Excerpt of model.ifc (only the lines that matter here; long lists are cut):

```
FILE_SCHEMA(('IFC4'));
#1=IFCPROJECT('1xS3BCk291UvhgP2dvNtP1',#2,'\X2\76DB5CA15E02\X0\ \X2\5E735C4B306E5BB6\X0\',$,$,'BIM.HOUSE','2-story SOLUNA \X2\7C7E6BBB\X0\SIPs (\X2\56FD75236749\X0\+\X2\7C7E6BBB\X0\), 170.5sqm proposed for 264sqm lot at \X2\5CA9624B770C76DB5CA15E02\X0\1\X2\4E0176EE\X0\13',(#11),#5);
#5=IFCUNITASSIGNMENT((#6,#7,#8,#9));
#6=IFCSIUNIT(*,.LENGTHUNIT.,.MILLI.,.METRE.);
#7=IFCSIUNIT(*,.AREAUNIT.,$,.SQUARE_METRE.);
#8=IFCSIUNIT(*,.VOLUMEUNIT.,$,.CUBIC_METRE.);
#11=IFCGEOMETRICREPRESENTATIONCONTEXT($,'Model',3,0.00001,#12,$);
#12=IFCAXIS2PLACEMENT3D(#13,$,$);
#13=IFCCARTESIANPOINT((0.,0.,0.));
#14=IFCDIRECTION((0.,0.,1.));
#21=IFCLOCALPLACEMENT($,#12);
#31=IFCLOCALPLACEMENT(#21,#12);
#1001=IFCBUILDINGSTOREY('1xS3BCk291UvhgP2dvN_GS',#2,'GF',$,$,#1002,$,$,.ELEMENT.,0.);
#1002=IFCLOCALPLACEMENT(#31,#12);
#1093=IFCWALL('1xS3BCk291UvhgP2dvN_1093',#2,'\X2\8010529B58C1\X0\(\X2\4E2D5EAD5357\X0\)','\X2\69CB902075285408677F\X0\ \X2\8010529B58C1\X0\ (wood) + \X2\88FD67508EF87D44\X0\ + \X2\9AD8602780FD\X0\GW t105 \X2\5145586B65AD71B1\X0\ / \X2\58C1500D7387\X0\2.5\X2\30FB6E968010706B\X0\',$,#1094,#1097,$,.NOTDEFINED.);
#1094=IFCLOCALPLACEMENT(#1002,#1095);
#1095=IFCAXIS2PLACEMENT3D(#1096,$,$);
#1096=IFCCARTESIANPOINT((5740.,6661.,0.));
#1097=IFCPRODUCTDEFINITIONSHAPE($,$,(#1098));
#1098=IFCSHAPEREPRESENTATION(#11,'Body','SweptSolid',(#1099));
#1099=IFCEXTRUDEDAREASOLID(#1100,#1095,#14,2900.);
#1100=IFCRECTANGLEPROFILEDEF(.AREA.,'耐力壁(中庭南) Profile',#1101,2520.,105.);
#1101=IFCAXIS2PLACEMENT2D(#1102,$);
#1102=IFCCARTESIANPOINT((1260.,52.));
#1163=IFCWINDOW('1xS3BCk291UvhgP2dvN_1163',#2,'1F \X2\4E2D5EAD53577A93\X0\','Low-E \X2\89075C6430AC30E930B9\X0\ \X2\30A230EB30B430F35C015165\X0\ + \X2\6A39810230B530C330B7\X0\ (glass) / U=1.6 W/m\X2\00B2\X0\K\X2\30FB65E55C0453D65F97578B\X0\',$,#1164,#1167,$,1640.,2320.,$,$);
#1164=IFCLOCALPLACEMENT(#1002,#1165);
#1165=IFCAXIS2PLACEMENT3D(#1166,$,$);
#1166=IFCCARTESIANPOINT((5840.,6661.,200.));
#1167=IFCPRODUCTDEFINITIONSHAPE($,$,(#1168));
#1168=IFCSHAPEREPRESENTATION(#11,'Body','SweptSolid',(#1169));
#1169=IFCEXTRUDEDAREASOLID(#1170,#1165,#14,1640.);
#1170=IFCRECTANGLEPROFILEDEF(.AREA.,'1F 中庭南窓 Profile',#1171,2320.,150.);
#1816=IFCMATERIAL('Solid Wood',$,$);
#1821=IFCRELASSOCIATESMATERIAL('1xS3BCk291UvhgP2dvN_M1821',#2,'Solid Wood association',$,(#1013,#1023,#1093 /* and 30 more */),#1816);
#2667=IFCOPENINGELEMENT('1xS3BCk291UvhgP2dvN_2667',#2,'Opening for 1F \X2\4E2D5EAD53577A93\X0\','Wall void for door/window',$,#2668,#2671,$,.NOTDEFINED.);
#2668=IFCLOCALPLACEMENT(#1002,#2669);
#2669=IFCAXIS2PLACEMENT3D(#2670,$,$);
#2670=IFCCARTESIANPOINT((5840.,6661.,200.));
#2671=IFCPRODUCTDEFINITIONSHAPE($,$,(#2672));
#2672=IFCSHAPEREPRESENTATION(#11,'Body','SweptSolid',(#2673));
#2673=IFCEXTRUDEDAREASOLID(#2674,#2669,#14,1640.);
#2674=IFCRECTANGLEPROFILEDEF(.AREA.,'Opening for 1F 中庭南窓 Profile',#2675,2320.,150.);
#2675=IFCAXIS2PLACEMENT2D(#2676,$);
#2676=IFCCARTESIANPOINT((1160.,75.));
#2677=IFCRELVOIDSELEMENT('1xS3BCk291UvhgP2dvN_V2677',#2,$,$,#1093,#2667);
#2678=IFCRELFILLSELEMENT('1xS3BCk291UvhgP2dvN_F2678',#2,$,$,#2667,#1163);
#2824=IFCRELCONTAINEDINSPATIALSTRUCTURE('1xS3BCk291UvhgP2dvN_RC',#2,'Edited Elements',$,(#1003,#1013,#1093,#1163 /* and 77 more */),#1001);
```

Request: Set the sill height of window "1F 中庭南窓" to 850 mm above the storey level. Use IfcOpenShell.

```python
import numpy as np
import ifcopenshell
import ifcopenshell.api.geometry
import ifcopenshell.geom
import ifcopenshell.util.element
import ifcopenshell.util.placement
import ifcopenshell.util.shape
import ifcopenshell.util.unit

model = ifcopenshell.open("model.ifc")
unit_scale = ifcopenshell.util.unit.calculate_unit_scale(model)

window = model.by_guid("1xS3BCk291UvhgP2dvN_1163")
opening = window.FillsVoids[0].RelatingOpeningElement
storey = ifcopenshell.util.element.get_container(window, ifc_class="IfcBuildingStorey")
level = ifcopenshell.util.placement.get_local_placement(storey.ObjectPlacement)[2, 3]

# The opening's origin need not be at the sill, so measure its lowest point.
shape = ifcopenshell.geom.create_shape(ifcopenshell.geom.settings(), opening)
bottom = ifcopenshell.util.shape.get_shape_bottom_elevation(shape, shape.geometry) / unit_scale
dz = level + 850.0 - bottom

shift = np.array([0.0, 0.0, dz])
# The window is not placed relative to its opening, so move both.
for product in (opening, window):
    matrix = ifcopenshell.util.placement.get_local_placement(product.ObjectPlacement)
    matrix[:3, 3] += shift
    ifcopenshell.api.geometry.edit_object_placement(model, product=product, matrix=matrix, is_si=False)

print(f"moved by {dz * unit_scale:+.3f} m")

model.write("model_updated.ifc")
```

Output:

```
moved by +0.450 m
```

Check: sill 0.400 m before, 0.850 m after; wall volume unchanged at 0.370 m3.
